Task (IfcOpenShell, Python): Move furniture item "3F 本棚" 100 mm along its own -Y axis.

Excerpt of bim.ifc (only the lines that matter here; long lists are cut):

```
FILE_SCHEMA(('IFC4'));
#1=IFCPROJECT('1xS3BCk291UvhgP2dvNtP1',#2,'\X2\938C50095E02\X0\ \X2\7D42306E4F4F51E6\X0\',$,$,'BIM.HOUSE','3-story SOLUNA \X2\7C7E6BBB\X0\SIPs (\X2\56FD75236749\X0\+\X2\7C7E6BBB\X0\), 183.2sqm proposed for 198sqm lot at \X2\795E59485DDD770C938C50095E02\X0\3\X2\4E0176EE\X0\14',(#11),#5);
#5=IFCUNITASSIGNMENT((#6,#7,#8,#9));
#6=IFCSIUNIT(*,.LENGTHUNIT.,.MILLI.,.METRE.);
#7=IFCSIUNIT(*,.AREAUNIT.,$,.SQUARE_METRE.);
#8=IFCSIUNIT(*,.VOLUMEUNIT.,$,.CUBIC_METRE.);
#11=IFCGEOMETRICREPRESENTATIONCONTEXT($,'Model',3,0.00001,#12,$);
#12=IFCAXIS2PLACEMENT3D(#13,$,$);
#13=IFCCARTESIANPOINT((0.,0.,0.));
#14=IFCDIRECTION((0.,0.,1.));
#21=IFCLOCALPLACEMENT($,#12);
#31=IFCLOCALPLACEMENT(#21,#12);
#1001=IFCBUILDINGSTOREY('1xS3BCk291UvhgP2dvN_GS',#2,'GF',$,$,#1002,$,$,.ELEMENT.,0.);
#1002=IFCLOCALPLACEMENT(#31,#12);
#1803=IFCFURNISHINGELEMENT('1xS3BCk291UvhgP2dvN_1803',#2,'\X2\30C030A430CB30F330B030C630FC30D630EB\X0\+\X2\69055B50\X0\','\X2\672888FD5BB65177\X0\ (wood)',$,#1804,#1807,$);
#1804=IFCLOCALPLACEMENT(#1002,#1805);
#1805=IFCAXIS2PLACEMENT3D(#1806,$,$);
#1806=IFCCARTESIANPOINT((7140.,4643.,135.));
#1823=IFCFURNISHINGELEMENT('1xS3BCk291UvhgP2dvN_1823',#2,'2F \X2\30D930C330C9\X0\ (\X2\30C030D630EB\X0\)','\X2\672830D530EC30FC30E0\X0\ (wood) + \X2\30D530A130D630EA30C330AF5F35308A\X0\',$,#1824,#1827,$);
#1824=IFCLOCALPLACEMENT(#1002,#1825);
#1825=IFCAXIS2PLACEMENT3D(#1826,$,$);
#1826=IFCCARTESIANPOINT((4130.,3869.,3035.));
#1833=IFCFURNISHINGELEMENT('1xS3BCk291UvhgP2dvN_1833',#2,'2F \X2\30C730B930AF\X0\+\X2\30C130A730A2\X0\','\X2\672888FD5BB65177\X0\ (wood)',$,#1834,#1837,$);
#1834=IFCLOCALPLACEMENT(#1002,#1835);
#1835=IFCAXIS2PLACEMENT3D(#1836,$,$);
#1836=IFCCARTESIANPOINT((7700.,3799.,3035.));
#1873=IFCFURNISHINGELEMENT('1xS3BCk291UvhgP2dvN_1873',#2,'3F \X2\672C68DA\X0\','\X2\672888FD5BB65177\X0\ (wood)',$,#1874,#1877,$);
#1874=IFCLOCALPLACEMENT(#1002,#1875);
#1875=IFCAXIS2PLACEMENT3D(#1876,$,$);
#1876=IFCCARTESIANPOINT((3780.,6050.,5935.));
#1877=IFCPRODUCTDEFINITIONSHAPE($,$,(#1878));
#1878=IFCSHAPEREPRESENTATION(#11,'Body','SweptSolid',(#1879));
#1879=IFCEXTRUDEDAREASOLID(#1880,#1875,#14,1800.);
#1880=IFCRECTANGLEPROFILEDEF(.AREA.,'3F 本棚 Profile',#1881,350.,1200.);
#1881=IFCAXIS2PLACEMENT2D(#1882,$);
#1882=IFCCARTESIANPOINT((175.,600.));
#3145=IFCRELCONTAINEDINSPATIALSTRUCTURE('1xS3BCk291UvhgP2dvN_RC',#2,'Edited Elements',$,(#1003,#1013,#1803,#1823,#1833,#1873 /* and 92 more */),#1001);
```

```python
import ifcopenshell
import ifcopenshell.api.geometry
import ifcopenshell.util.placement
import ifcopenshell.util.unit

model = ifcopenshell.open("bim.ifc")
unit_scale = ifcopenshell.util.unit.calculate_unit_scale(model)

item = model.by_guid("1xS3BCk291UvhgP2dvN_1873")
matrix = ifcopenshell.util.placement.get_local_placement(item.ObjectPlacement)
matrix[:3, 3] -= matrix[:3, 1] * 0.1 / unit_scale
ifcopenshell.api.geometry.edit_object_placement(model, product=item, matrix=matrix, is_si=False)

print(ifcopenshell.util.placement.get_local_placement(item.ObjectPlacement).round(3) + 0.0)

model.write("bim_v2.ifc")
```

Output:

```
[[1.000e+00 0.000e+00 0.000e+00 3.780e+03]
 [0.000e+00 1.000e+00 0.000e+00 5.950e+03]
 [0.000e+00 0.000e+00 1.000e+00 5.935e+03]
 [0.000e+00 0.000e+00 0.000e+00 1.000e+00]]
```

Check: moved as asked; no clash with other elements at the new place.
